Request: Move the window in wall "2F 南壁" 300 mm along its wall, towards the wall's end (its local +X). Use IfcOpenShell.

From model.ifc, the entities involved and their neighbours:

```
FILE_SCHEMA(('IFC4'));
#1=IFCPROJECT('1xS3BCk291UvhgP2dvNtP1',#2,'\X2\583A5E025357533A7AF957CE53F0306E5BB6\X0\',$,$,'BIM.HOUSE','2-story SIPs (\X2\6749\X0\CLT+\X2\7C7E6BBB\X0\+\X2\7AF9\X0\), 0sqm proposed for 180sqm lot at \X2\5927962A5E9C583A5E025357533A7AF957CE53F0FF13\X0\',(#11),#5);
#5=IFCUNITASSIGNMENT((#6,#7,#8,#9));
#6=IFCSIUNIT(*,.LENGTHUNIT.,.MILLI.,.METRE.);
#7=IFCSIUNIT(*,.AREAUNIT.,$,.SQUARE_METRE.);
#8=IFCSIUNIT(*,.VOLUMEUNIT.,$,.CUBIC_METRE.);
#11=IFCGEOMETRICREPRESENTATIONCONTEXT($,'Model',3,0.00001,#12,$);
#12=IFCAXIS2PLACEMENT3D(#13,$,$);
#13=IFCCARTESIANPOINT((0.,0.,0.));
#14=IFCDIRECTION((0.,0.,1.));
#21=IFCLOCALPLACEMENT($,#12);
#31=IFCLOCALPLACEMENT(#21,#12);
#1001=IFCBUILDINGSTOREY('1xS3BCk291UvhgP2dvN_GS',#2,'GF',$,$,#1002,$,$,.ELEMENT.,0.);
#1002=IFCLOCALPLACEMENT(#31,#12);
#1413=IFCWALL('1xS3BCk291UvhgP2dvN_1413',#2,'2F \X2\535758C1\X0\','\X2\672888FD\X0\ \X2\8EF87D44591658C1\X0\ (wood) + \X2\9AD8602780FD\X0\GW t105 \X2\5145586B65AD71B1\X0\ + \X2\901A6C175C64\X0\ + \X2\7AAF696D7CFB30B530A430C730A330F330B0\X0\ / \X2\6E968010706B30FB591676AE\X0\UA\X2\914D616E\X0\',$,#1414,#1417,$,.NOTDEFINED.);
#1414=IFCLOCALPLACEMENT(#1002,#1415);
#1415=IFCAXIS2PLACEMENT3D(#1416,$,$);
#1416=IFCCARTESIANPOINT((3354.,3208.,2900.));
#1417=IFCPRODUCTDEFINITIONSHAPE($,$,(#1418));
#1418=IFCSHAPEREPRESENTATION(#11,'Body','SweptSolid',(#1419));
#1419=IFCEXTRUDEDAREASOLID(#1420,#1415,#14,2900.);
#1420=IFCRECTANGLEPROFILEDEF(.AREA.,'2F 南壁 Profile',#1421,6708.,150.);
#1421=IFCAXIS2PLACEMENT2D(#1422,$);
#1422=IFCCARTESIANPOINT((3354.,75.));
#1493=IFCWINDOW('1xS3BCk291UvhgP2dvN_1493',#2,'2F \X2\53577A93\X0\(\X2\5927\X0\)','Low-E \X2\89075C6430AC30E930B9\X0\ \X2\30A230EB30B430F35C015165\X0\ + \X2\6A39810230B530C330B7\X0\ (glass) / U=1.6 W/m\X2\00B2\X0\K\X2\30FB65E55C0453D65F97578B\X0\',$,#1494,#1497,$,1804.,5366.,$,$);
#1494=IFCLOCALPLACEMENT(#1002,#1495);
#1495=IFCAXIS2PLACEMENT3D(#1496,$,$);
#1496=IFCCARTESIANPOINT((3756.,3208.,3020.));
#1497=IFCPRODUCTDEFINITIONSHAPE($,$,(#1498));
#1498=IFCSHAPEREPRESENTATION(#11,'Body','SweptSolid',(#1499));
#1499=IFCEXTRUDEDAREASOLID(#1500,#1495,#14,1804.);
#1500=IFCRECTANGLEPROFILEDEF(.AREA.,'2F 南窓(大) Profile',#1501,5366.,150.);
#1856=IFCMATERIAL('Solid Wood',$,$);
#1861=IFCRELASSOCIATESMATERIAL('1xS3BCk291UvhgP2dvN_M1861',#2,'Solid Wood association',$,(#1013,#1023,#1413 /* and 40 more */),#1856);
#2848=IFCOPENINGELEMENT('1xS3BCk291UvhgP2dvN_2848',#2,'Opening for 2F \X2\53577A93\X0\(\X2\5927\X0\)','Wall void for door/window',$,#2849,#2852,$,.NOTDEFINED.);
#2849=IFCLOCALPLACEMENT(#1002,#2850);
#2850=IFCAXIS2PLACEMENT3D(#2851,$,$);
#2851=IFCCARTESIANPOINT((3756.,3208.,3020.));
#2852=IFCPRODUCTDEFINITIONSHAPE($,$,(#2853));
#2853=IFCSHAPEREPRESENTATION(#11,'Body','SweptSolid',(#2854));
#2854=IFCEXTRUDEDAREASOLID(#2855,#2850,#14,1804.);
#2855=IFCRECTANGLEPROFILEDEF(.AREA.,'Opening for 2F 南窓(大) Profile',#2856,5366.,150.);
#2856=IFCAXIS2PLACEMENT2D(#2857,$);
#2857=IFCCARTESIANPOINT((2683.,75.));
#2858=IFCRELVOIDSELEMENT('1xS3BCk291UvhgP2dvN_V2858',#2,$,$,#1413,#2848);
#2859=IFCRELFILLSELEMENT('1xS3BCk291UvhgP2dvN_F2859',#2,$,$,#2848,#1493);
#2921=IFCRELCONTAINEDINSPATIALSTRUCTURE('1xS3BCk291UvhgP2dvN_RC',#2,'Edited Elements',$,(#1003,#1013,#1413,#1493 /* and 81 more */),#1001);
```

```python
import ifcopenshell
import ifcopenshell.api.geometry
import ifcopenshell.util.placement

model = ifcopenshell.open("model.ifc")

window = model.by_id(1493)
opening = window.FillsVoids[0].RelatingOpeningElement
wall = opening.VoidsElements[0].RelatingBuildingElement

wall_matrix = ifcopenshell.util.placement.get_local_placement(wall.ObjectPlacement)
shift = wall_matrix[:3, 0] * 300.0
before = ifcopenshell.util.placement.get_local_placement(window.ObjectPlacement)[:3, 3].copy()

# The window is not placed relative to its opening, so move both.
for product in (opening, window):
    matrix = ifcopenshell.util.placement.get_local_placement(product.ObjectPlacement)
    matrix[:3, 3] += shift
    ifcopenshell.api.geometry.edit_object_placement(model, product=product, matrix=matrix, is_si=False)

after = ifcopenshell.util.placement.get_local_placement(window.ObjectPlacement)[:3, 3]
print("window moved by", (after - before).round(3) + 0.0)

model.write("model-out.ifc")
```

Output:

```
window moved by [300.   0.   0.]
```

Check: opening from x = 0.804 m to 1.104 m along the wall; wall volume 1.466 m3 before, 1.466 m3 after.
